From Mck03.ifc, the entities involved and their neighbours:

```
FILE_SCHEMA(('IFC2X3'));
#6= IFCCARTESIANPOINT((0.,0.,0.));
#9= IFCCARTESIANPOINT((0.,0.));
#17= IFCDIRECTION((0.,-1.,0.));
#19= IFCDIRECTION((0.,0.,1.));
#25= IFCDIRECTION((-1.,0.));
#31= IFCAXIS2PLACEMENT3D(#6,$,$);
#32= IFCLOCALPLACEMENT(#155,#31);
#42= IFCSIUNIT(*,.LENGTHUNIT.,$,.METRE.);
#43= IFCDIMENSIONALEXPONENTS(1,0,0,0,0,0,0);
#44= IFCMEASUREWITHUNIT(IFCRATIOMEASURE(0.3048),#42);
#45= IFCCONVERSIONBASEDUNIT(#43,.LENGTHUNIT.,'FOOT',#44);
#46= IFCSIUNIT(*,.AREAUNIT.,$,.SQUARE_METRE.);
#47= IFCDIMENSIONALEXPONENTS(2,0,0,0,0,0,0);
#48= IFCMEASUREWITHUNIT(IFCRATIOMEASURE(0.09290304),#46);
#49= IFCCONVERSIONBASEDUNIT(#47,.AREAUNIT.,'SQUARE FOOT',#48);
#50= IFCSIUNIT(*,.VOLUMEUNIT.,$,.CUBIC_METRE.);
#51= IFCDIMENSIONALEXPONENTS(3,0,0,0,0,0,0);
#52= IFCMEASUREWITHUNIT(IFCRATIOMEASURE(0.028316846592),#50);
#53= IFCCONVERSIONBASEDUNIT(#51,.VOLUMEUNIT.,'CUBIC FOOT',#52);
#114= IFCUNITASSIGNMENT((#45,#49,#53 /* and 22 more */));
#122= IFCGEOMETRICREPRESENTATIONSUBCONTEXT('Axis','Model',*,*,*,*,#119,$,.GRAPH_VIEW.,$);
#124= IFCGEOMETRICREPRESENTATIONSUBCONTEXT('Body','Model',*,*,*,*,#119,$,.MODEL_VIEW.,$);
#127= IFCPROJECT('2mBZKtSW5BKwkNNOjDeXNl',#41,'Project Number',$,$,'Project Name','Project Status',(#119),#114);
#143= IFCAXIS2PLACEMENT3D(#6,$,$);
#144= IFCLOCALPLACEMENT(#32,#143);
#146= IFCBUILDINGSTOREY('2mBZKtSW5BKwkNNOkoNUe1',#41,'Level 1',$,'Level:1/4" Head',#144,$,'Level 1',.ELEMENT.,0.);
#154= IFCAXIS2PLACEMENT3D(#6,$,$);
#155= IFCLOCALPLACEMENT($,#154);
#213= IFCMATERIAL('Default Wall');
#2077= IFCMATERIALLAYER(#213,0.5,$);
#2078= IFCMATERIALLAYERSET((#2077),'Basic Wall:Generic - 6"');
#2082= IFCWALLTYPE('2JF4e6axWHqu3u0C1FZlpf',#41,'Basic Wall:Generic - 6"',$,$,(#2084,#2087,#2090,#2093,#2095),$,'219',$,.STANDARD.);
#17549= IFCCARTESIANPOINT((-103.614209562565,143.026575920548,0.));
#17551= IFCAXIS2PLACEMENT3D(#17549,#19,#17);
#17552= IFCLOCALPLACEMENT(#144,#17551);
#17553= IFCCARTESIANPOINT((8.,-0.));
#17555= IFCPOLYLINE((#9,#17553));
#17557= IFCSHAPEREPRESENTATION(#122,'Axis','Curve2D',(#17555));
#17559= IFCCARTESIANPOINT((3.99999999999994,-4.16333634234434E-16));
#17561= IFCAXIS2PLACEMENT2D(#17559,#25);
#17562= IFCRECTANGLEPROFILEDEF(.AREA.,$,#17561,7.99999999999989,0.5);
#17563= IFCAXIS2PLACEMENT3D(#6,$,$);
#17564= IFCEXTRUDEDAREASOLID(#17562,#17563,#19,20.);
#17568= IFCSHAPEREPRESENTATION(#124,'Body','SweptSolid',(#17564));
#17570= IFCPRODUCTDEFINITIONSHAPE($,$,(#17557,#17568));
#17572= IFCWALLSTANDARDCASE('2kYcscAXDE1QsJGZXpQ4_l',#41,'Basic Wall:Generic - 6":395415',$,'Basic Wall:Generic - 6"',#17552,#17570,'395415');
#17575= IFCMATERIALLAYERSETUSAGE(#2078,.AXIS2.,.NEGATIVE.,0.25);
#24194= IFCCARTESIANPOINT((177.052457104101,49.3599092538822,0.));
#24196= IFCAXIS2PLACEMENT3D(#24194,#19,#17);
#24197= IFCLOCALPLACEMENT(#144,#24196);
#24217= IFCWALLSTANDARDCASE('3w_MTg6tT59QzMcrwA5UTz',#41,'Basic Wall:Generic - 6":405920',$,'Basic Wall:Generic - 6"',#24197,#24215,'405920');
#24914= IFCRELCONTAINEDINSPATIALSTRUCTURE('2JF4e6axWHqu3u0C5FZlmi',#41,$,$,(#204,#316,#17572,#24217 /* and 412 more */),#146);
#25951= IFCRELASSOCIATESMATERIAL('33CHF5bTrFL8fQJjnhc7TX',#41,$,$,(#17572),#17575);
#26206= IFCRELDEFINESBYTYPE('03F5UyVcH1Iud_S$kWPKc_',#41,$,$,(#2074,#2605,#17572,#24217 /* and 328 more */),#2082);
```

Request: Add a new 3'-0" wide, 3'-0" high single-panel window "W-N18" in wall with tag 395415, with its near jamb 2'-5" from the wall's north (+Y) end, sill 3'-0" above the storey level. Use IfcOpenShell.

```python
import numpy as np
import ifcopenshell
import ifcopenshell.api.feature
import ifcopenshell.api.geometry
import ifcopenshell.api.root
import ifcopenshell.api.spatial
import ifcopenshell.api.type
import ifcopenshell.geom
import ifcopenshell.util.element
import ifcopenshell.util.placement
import ifcopenshell.util.representation
import ifcopenshell.util.shape
import ifcopenshell.util.unit

model = ifcopenshell.open("Mck03.ifc")
unit_scale = ifcopenshell.util.unit.calculate_unit_scale(model)
settings = ifcopenshell.geom.settings()


def volume(element):
    """Net volume in cubic metres, openings subtracted."""
    shape = ifcopenshell.geom.create_shape(settings, element)
    return ifcopenshell.util.shape.get_volume(shape.geometry)


wall = model.by_guid("2kYcscAXDE1QsJGZXpQ4_l")
storey = ifcopenshell.util.element.get_container(wall, ifc_class="IfcBuildingStorey")
context = ifcopenshell.util.representation.get_context(model, "Model", "Body", "MODEL_VIEW")
before = volume(wall)

width, height, from_end, sill = 0.9144, 0.9144, 0.7366, 0.9144  # metres

# The wall runs along its own X axis, and the end named is its -X end.
wall_shape = ifcopenshell.geom.create_shape(settings, wall)
x, y, z = ifcopenshell.util.shape.get_vertices(wall_shape.geometry).T
start = x.min() + from_end
face, thickness = float(y.min()), float(y.max() - y.min())
wall_matrix = ifcopenshell.util.placement.get_local_placement(wall.ObjectPlacement)
level = ifcopenshell.util.placement.get_local_placement(storey.ObjectPlacement)[2, 3]


def in_wall(x, y):
    """Placement at x, y metres in the wall's axes, at sill height."""
    matrix = wall_matrix.copy()
    matrix[:, 3] = wall_matrix @ np.array([x / unit_scale, y / unit_scale, 0.0, 1.0])
    matrix[2, 3] = level + sill / unit_scale
    return matrix


# Opening: a box that overshoots both wall faces by 50 mm.
opening = ifcopenshell.api.root.create_entity(model, ifc_class="IfcOpeningElement")
box = ifcopenshell.api.geometry.add_wall_representation(
    model, context=context, length=width, height=height, thickness=thickness + 0.1
)
ifcopenshell.api.geometry.assign_representation(model, product=opening, representation=box)
ifcopenshell.api.geometry.edit_object_placement(model, product=opening, matrix=in_wall(start, face - 0.05), is_si=False)
ifcopenshell.api.feature.add_feature(model, feature=opening, element=wall)

window = ifcopenshell.api.root.create_entity(model, ifc_class="IfcWindow", name="W-N18")
window.OverallWidth, window.OverallHeight = width / unit_scale, height / unit_scale
body = ifcopenshell.api.geometry.add_window_representation(
    model,
    context=context,
    overall_width=window.OverallWidth,
    overall_height=window.OverallHeight,
    partition_type="SINGLE_PANEL",
)
ifcopenshell.api.geometry.assign_representation(model, product=window, representation=body)
ifcopenshell.api.spatial.assign_container(model, products=[window], relating_structure=storey)
fills = ifcopenshell.api.feature.add_filling(model, opening=opening, element=window)
fills.OwnerHistory = window.OwnerHistory  # required in IFC2X3

# IFC2X3 keeps the operation on the window style.
style = ifcopenshell.api.root.create_entity(model, ifc_class="IfcWindowStyle", name="W-N18")
style.OperationType, style.ConstructionType = "SINGLE_PANEL", "NOTDEFINED"
style.ParameterTakesPrecedence = style.Sizeable = False
ifcopenshell.api.type.assign_type(model, related_objects=[window], relating_type=style)

# Centre the window in the wall's thickness.
ifcopenshell.api.geometry.edit_object_placement(model, product=window, matrix=in_wall(start, face), is_si=False)
window_shape = ifcopenshell.geom.create_shape(settings, window)
depth = ifcopenshell.util.shape.get_vertices(window_shape.geometry)[:, 1]
offset = face + thickness / 2 - (depth.min() + depth.max()) / 2
ifcopenshell.api.geometry.edit_object_placement(model, product=window, matrix=in_wall(start, offset), is_si=False)

after = volume(wall)

print(f"wall volume {before:.3f} -> {after:.3f} m3")

model.write("Mck03_updated.ifc")
```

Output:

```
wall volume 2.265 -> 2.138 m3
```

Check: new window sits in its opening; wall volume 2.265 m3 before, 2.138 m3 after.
